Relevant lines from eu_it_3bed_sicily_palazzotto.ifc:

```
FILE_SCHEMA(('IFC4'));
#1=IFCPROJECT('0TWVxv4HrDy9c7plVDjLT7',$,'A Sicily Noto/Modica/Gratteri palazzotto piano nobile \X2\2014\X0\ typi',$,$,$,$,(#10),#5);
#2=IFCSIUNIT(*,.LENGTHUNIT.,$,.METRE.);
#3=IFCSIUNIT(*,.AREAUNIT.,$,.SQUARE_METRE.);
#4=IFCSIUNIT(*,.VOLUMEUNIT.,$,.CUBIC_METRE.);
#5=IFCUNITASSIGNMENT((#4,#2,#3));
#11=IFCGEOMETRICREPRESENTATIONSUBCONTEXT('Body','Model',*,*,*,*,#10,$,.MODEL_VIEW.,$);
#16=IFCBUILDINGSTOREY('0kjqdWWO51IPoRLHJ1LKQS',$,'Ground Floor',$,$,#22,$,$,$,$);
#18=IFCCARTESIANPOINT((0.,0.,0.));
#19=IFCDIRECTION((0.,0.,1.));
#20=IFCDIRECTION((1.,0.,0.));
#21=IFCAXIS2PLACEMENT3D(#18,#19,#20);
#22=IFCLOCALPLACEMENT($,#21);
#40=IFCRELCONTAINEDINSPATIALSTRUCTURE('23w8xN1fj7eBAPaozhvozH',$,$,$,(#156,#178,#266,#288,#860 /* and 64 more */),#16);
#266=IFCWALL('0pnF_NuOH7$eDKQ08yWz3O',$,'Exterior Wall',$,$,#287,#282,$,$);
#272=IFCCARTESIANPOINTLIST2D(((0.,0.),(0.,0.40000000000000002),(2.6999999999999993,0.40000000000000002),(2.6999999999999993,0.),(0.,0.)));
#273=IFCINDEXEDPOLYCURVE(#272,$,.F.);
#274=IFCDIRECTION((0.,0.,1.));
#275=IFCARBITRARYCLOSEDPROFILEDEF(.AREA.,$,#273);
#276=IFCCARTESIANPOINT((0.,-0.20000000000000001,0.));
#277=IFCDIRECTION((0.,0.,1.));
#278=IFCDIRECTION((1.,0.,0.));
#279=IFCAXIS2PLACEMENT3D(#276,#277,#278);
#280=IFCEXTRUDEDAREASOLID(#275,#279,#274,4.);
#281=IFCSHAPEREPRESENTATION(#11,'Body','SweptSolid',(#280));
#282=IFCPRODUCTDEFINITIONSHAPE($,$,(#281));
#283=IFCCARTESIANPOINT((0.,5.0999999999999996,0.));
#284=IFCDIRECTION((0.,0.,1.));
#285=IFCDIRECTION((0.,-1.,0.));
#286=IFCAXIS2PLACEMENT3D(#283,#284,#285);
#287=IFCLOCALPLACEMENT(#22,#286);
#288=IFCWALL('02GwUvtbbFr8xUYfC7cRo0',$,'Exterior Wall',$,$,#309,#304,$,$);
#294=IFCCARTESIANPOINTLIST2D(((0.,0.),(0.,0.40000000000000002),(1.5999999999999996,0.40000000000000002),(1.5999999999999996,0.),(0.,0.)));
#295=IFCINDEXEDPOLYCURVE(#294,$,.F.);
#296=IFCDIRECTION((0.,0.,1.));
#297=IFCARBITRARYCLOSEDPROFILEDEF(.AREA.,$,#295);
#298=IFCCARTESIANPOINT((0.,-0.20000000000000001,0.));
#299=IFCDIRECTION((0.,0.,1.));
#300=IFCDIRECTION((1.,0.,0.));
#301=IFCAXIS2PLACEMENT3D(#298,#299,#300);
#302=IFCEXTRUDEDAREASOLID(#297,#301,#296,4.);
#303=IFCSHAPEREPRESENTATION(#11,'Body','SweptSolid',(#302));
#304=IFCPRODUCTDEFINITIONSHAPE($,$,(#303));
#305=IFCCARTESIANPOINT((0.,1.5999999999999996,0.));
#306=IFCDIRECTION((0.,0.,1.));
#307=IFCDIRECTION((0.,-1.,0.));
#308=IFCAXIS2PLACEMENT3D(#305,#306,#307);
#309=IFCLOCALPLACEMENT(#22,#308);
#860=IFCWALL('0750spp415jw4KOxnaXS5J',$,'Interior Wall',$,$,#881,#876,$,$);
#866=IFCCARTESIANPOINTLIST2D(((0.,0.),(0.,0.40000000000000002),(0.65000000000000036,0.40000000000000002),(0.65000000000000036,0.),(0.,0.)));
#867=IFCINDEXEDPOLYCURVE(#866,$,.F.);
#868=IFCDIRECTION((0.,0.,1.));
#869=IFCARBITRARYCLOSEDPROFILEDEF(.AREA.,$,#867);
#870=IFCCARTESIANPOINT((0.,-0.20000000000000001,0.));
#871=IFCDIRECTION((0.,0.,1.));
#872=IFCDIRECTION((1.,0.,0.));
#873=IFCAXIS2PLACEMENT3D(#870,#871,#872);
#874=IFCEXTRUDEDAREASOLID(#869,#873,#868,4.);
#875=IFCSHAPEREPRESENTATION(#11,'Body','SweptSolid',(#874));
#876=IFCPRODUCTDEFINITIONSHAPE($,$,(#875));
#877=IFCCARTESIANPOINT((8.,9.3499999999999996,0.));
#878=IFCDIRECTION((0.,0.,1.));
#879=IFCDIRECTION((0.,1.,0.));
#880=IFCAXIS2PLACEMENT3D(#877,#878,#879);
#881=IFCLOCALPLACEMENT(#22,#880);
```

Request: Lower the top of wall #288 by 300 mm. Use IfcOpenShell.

```python
import ifcopenshell
import ifcopenshell.geom
import ifcopenshell.util.representation
import ifcopenshell.util.shape
import ifcopenshell.util.unit

model = ifcopenshell.open("eu_it_3bed_sicily_palazzotto.ifc")
unit_scale = ifcopenshell.util.unit.calculate_unit_scale(model)
settings = ifcopenshell.geom.settings()


def volume(element):
    """Net volume in cubic metres, openings subtracted."""
    shape = ifcopenshell.geom.create_shape(settings, element)
    return ifcopenshell.util.shape.get_volume(shape.geometry)


wall = model.by_id(288)
before = volume(wall)

body = ifcopenshell.util.representation.get_representation(wall, "Model", "Body")
solid = body.Items[0]
old_height = solid.Depth
solid.Depth -= 0.3 / unit_scale
after = volume(wall)

print(f"height {old_height:g} -> {solid.Depth:g}, volume {before:.3f} -> {after:.3f} m3")

model.write("eu_it_3bed_sicily_palazzotto_edited.ifc")
```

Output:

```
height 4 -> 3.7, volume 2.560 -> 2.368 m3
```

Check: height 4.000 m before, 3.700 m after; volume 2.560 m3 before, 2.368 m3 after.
